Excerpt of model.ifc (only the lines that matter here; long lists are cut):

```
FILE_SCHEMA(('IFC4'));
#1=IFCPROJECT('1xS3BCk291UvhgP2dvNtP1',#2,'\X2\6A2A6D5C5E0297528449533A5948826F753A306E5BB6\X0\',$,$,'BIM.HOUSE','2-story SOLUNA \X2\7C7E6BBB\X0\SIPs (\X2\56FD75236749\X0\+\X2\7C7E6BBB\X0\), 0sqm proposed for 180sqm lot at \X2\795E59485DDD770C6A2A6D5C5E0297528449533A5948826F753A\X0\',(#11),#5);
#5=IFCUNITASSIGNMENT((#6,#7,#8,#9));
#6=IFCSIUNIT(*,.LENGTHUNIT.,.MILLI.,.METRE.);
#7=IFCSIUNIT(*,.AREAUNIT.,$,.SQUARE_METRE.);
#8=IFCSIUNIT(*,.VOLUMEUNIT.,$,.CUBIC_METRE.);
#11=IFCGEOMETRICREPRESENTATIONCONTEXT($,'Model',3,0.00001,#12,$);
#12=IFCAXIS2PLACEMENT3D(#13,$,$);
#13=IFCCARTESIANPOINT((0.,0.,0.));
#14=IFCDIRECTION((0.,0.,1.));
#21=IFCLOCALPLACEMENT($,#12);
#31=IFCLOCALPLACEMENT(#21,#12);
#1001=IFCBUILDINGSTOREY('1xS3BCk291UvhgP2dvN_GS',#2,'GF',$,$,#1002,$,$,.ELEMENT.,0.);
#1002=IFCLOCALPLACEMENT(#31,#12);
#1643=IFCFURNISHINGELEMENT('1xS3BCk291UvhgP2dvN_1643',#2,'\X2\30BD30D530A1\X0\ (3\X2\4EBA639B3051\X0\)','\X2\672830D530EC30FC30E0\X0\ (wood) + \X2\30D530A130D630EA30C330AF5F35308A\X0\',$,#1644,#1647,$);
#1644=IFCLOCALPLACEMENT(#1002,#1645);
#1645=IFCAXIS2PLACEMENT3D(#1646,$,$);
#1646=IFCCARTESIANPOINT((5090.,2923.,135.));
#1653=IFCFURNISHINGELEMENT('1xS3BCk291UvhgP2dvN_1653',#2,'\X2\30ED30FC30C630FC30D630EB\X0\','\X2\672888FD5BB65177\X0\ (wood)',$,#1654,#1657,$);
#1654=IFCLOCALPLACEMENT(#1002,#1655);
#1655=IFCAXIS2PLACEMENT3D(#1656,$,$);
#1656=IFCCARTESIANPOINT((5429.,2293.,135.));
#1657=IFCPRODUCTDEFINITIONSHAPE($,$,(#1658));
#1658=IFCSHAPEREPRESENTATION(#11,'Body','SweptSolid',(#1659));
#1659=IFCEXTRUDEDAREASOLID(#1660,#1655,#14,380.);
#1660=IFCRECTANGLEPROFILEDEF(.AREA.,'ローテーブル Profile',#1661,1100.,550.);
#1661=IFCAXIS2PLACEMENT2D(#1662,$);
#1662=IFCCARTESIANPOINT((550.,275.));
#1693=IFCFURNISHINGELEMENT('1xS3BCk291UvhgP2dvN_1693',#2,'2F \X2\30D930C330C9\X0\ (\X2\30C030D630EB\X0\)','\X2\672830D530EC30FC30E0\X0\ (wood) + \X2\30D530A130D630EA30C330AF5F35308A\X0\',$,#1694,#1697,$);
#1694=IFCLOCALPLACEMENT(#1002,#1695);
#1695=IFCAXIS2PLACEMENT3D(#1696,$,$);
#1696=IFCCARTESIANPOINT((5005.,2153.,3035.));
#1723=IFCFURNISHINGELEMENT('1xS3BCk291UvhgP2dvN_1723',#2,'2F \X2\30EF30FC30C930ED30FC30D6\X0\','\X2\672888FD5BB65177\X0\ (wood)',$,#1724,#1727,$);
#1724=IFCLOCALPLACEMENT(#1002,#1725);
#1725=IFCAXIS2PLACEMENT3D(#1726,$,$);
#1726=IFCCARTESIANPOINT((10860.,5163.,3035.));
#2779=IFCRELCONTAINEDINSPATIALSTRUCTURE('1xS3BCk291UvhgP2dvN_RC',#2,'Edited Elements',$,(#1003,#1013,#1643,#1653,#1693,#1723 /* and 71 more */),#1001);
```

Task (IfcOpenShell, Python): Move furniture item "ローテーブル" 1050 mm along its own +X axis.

```python
import ifcopenshell
import ifcopenshell.api.geometry
import ifcopenshell.util.placement
import ifcopenshell.util.unit

model = ifcopenshell.open("model.ifc")
unit_scale = ifcopenshell.util.unit.calculate_unit_scale(model)

item = model.by_id(1653)
matrix = ifcopenshell.util.placement.get_local_placement(item.ObjectPlacement)
matrix[:3, 3] += matrix[:3, 0] * 1.05 / unit_scale
ifcopenshell.api.geometry.edit_object_placement(model, product=item, matrix=matrix, is_si=False)

print(ifcopenshell.util.placement.get_local_placement(item.ObjectPlacement).round(3) + 0.0)

model.write("model_rev.ifc")
```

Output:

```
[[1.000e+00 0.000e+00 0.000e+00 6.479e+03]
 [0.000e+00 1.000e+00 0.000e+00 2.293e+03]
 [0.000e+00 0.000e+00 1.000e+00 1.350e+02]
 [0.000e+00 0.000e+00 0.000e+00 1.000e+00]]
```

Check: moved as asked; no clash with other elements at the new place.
